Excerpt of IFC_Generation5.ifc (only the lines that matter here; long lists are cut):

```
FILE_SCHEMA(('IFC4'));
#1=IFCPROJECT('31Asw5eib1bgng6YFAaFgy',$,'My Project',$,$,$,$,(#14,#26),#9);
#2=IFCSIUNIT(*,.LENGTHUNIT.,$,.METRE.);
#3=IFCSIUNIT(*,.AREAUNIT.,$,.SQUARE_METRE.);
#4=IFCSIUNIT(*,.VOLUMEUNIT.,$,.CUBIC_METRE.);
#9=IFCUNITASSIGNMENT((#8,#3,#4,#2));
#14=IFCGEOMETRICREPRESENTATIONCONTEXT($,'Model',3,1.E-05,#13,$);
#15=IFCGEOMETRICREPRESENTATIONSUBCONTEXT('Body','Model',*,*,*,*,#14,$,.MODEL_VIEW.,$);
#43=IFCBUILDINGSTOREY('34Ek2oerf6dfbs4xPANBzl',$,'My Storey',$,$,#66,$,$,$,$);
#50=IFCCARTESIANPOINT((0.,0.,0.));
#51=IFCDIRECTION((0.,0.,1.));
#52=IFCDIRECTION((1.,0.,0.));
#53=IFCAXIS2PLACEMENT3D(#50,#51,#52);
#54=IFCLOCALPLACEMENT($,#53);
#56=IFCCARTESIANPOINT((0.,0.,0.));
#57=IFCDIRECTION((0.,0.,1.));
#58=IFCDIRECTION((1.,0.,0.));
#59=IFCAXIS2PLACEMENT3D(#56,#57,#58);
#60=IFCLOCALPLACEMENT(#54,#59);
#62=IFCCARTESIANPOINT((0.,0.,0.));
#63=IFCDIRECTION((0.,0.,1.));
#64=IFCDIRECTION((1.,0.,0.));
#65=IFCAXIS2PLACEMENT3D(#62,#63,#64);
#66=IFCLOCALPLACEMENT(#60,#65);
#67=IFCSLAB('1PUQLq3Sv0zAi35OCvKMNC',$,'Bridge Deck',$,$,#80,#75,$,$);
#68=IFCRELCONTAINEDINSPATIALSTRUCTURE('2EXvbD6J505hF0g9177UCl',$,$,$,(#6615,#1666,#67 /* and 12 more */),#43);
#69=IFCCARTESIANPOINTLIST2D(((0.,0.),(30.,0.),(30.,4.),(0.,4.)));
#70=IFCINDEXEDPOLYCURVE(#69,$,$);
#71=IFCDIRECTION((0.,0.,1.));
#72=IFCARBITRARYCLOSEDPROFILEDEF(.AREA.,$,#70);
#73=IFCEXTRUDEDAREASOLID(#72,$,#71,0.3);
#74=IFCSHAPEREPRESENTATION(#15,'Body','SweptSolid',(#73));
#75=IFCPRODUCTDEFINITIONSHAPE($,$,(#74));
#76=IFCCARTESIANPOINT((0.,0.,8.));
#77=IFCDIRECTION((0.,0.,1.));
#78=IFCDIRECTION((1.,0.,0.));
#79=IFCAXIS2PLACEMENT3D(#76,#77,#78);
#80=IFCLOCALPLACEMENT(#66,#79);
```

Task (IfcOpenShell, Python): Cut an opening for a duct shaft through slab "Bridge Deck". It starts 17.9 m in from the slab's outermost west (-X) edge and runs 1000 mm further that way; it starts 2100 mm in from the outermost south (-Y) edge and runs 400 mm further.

```python
import numpy as np
import ifcopenshell
import ifcopenshell.api.feature
import ifcopenshell.api.geometry
import ifcopenshell.api.root
import ifcopenshell.geom
import ifcopenshell.util.placement
import ifcopenshell.util.representation
import ifcopenshell.util.shape
import ifcopenshell.util.unit

model = ifcopenshell.open("IFC_Generation5.ifc")
unit_scale = ifcopenshell.util.unit.calculate_unit_scale(model)
settings = ifcopenshell.geom.settings()


def volume(element):
    """Net volume in cubic metres, openings subtracted."""
    shape = ifcopenshell.geom.create_shape(settings, element)
    return ifcopenshell.util.shape.get_volume(shape.geometry)


slab = model.by_id(67)
before = volume(slab)

# Extent in the slab's own axes, in metres. The edges named are its -X and -Y sides.
slab_shape = ifcopenshell.geom.create_shape(settings, slab)
vertices = ifcopenshell.util.shape.get_vertices(slab_shape.geometry)
x_min, y_min, bottom = vertices.min(axis=0)
top = vertices[:, 2].max()

opening = ifcopenshell.api.root.create_entity(model, ifc_class="IfcOpeningElement", name="Duct shaft opening", predefined_type="OPENING")
context = ifcopenshell.util.representation.get_context(model, "Model", "Body", "MODEL_VIEW")
width, depth = 1, 0.4
outline = [(0.0, 0.0), (width, 0.0), (width, depth), (0.0, depth), (0.0, 0.0)]
# Overshoot both faces by 50 mm so the cut is clean.
shape = ifcopenshell.api.geometry.add_slab_representation(
    model, context=context, depth=top - bottom + 0.1, polyline=outline
)
ifcopenshell.api.geometry.assign_representation(model, product=opening, representation=shape)

matrix = ifcopenshell.util.placement.get_local_placement(slab.ObjectPlacement)
matrix[:, 3] = matrix @ np.append(np.array([x_min + 17.9, y_min + 2.1, bottom - 0.05]) / unit_scale, 1.0)
ifcopenshell.api.geometry.edit_object_placement(model, product=opening, matrix=matrix, is_si=False)
ifcopenshell.api.feature.add_feature(model, feature=opening, element=slab)

after = volume(slab)

print(f"slab volume {before:.3f} -> {after:.3f} m3")

model.write("IFC_Generation5_rev.ifc")
```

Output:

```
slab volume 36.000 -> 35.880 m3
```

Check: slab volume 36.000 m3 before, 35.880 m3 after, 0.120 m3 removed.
